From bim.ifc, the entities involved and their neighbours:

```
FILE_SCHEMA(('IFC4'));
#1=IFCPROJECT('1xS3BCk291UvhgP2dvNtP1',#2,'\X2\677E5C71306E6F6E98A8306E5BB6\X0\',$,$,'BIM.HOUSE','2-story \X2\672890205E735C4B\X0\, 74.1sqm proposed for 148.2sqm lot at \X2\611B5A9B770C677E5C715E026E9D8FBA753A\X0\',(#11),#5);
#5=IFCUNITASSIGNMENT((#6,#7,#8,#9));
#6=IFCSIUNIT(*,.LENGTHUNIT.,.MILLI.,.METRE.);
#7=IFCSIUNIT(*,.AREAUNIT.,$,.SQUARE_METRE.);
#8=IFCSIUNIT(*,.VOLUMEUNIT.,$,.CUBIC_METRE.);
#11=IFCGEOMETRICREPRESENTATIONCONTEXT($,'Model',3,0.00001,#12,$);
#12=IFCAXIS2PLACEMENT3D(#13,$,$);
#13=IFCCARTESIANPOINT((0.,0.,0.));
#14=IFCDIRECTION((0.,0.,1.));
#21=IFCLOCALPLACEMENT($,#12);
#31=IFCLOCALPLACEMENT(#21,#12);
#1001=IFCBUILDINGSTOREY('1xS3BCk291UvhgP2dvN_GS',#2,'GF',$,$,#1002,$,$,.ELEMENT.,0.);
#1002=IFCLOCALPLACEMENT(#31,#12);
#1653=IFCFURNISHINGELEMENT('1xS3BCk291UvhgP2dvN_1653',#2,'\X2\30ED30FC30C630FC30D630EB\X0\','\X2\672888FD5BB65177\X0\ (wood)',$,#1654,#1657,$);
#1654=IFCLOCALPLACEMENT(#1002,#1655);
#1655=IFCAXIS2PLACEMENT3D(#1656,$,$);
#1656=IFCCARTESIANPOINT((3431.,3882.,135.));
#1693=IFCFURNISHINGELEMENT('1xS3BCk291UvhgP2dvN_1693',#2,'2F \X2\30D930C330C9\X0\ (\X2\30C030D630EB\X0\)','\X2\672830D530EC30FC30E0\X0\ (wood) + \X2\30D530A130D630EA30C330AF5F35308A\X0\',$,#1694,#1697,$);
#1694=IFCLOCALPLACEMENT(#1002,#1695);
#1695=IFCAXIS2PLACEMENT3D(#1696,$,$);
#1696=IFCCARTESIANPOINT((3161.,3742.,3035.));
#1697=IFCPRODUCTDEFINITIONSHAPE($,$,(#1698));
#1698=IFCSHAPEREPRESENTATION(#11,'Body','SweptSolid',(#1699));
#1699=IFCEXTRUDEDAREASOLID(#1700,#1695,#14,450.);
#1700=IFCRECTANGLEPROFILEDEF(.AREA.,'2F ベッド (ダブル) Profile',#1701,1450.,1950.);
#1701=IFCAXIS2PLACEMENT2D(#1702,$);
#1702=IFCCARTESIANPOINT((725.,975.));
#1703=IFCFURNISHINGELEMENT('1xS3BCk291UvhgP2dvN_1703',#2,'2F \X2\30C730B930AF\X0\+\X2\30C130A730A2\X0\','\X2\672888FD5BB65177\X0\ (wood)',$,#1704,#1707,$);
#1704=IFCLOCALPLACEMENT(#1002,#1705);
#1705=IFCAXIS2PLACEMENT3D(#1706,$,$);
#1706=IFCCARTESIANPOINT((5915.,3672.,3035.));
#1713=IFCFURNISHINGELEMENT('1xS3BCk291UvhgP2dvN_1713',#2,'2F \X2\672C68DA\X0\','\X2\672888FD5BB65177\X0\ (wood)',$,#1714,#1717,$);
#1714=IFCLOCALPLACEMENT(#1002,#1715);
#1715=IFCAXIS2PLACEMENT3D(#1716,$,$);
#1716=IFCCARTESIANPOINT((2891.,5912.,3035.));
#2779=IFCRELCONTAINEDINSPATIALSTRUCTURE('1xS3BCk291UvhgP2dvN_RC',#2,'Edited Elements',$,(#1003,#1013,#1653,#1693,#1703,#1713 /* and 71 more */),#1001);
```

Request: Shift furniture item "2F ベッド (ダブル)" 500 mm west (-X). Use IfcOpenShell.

```python
import ifcopenshell
import ifcopenshell.api.geometry
import ifcopenshell.util.placement
import ifcopenshell.util.unit

model = ifcopenshell.open("bim.ifc")
unit_scale = ifcopenshell.util.unit.calculate_unit_scale(model)

item = model.by_id(1693)
matrix = ifcopenshell.util.placement.get_local_placement(item.ObjectPlacement)
matrix[0, 3] -= 0.5 / unit_scale
ifcopenshell.api.geometry.edit_object_placement(model, product=item, matrix=matrix, is_si=False)

print(ifcopenshell.util.placement.get_local_placement(item.ObjectPlacement).round(3) + 0.0)

model.write("bim_updated.ifc")
```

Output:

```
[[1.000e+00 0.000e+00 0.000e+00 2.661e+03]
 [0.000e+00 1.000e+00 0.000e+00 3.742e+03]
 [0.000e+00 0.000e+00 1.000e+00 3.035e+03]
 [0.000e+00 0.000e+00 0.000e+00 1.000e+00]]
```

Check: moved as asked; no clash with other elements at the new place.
